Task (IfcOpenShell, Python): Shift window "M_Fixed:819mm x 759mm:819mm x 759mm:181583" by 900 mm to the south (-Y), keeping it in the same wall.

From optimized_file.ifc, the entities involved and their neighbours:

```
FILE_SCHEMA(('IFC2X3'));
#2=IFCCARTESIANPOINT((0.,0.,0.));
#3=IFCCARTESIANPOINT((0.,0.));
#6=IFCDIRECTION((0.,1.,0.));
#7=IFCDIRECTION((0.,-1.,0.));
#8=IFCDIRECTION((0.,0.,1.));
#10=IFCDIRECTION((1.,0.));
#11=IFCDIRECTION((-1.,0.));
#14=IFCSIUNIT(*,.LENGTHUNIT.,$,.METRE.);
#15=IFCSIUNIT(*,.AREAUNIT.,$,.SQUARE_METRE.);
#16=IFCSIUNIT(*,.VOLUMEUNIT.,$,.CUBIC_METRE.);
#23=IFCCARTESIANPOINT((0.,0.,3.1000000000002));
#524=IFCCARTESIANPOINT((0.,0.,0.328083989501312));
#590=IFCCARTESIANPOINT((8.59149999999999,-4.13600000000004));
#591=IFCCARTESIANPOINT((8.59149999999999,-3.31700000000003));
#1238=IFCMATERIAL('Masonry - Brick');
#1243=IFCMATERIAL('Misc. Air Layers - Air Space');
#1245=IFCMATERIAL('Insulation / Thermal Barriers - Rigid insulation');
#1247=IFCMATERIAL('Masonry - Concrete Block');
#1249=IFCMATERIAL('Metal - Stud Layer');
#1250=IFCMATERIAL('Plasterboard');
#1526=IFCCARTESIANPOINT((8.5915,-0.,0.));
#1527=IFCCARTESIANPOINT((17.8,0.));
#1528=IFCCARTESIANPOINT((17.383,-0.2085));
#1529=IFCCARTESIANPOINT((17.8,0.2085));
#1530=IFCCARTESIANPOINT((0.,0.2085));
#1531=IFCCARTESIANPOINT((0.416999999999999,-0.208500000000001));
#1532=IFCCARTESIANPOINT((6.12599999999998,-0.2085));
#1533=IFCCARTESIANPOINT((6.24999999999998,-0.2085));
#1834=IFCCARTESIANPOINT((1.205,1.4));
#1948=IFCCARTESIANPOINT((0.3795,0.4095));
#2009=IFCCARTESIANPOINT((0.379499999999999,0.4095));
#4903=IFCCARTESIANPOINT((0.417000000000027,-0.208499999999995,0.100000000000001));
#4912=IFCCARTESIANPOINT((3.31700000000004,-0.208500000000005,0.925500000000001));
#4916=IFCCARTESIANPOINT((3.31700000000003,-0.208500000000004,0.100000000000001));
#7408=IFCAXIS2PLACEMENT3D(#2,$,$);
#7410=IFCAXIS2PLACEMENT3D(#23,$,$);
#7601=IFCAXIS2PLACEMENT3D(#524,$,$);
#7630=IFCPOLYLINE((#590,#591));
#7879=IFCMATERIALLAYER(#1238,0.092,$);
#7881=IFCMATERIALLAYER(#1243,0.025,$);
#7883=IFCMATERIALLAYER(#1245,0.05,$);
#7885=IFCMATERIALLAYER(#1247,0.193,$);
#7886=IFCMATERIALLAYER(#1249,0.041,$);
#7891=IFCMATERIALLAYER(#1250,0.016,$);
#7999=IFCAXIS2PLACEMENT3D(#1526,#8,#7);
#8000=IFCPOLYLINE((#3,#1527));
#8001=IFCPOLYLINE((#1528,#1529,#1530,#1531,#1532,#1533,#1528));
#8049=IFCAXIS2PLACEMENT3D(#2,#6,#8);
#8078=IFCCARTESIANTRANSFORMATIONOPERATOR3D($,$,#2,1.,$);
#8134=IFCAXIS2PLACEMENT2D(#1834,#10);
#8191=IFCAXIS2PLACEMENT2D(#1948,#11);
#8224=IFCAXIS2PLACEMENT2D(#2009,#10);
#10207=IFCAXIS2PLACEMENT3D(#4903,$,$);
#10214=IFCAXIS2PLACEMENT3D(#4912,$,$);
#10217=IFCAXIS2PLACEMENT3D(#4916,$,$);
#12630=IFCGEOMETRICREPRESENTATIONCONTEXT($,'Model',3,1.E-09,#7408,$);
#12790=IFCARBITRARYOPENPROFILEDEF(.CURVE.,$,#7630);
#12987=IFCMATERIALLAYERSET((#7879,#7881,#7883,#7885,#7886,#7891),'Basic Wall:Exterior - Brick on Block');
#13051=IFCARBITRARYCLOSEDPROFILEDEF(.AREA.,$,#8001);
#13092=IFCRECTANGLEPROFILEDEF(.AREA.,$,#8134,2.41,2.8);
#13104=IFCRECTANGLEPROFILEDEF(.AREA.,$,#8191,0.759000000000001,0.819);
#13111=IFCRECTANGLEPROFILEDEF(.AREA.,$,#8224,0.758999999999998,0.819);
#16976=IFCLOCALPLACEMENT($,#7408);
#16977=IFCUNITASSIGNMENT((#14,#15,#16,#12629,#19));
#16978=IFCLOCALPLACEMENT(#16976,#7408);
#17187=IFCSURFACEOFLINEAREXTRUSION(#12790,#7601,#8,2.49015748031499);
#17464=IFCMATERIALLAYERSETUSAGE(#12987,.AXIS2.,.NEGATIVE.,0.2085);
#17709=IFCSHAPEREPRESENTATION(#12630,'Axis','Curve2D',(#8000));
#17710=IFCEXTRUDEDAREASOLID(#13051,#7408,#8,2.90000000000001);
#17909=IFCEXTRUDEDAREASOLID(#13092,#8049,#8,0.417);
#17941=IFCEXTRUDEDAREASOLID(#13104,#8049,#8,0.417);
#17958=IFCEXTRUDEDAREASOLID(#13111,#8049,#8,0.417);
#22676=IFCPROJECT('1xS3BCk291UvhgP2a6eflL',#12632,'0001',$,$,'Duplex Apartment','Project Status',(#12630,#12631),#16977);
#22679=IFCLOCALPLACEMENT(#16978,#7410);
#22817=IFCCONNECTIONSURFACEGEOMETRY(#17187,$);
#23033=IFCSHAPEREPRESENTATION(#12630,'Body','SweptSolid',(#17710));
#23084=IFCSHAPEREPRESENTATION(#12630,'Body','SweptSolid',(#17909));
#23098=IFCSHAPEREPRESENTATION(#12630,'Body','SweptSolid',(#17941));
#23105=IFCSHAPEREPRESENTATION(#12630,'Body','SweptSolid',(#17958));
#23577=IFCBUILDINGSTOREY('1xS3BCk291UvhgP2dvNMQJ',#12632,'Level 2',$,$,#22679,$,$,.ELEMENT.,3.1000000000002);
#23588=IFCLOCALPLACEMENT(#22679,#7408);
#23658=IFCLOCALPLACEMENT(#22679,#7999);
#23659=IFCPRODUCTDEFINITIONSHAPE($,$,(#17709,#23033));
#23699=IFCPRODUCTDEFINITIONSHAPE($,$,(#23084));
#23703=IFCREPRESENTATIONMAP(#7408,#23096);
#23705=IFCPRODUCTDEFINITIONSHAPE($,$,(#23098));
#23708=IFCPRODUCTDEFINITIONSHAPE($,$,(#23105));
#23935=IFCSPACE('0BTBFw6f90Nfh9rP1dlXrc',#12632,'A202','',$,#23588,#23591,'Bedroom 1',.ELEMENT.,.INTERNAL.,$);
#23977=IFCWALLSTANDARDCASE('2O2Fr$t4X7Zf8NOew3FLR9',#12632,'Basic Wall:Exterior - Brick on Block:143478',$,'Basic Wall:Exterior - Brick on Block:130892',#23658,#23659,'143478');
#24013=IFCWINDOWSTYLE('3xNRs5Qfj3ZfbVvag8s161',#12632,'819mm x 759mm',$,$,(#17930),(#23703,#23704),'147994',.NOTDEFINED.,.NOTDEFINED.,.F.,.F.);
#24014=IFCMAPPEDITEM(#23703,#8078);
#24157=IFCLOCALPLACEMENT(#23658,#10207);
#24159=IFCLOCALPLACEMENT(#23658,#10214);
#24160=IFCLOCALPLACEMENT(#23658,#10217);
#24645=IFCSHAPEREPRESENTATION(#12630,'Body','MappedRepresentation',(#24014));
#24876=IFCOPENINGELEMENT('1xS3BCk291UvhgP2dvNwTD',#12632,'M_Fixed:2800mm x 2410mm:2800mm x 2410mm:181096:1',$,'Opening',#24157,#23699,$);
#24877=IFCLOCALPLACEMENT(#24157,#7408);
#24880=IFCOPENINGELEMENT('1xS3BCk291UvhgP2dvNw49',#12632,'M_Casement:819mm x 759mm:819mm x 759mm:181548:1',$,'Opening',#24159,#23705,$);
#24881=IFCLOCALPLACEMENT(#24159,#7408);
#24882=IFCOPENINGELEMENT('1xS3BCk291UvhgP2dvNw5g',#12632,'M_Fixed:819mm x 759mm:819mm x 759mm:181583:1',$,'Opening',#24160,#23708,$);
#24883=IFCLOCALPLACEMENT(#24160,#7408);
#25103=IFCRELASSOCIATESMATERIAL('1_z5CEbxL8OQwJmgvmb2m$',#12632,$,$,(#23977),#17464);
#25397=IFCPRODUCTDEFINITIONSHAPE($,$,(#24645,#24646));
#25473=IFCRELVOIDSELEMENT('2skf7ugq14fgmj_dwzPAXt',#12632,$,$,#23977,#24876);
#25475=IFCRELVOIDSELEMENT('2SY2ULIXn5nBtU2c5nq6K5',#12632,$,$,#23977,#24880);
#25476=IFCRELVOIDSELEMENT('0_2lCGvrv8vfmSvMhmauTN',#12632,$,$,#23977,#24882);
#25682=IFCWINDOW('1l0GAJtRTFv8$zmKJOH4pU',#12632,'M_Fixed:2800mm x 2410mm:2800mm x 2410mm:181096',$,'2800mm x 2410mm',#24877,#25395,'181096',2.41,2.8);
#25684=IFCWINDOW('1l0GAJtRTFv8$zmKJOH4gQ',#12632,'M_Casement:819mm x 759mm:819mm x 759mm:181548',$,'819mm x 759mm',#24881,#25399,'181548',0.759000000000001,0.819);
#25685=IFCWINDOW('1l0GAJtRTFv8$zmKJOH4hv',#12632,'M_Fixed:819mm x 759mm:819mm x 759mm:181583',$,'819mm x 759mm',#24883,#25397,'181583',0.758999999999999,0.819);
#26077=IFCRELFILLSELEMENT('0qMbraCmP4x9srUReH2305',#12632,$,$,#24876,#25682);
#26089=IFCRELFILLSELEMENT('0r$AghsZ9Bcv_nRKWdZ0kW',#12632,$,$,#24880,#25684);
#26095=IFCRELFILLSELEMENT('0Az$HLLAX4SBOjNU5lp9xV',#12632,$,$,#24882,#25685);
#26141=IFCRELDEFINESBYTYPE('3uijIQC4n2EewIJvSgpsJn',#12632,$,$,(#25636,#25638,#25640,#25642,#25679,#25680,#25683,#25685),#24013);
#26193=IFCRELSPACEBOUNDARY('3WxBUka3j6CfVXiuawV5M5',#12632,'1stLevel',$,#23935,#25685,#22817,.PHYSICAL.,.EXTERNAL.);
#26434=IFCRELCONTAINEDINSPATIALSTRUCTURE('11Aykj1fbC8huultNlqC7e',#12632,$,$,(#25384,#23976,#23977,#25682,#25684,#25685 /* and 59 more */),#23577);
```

```python
import numpy as np
import ifcopenshell
import ifcopenshell.api.geometry
import ifcopenshell.util.placement
import ifcopenshell.util.unit

model = ifcopenshell.open("optimized_file.ifc")
unit_scale = ifcopenshell.util.unit.calculate_unit_scale(model)

window = model.by_guid("1l0GAJtRTFv8$zmKJOH4hv")
opening = window.FillsVoids[0].RelatingOpeningElement
wall = opening.VoidsElements[0].RelatingBuildingElement

wall_matrix = ifcopenshell.util.placement.get_local_placement(wall.ObjectPlacement)
shift = wall_matrix[:3, 0] * 0.9 / unit_scale
before = ifcopenshell.util.placement.get_local_placement(window.ObjectPlacement)[:3, 3].copy()

# The window is placed relative to its opening, so it follows when the opening moves.
matrix = ifcopenshell.util.placement.get_local_placement(opening.ObjectPlacement)
matrix[:3, 3] += shift
ifcopenshell.api.geometry.edit_object_placement(
    model, product=opening, matrix=matrix, is_si=False, should_transform_children=True
)

# Space boundary surfaces are stored in each space's coordinates; move them too.
for rel in window.ProvidesBoundaries:
    if not rel.ConnectionGeometry:
        continue
    surface = rel.ConnectionGeometry.SurfaceOnRelatingElement
    space_matrix = ifcopenshell.util.placement.get_local_placement(rel.RelatingSpace.ObjectPlacement)
    point = np.array(surface.Position.Location.Coordinates) + space_matrix[:3, :3].T @ shift
    surface.Position = model.createIfcAxis2Placement3D(
        model.createIfcCartesianPoint(point.tolist()), surface.Position.Axis, surface.Position.RefDirection
    )

after = ifcopenshell.util.placement.get_local_placement(window.ObjectPlacement)[:3, 3]
print("window moved by", (after - before).round(3) + 0.0)

model.write("optimized_file-out.ifc")
```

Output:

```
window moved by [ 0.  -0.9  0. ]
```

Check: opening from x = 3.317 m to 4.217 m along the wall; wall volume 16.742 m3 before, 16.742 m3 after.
